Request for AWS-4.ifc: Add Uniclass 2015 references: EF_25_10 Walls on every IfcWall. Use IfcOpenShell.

First a look at what the model holds.

```python
import ifcopenshell

model = ifcopenshell.open("AWS-4.ifc")
print(model.schema)
print("classifications:", [c.Name for c in model.by_type("IfcClassification")])
for ifc_class in ("IfcDoor", "IfcRoof", "IfcStair", "IfcWall", "IfcWindow"):
    print(ifc_class, len(model.by_type(ifc_class)))
```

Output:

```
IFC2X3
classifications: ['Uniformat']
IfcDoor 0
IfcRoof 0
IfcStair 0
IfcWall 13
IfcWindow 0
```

```python
import ifcopenshell
import ifcopenshell.api.classification

model = ifcopenshell.open("AWS-4.ifc")

# IFC2X3 requires Source and Edition and has no link from the project to the system.
system = model.create_entity("IfcClassification", Source="NBS", Edition="2015", Name="Uniclass 2015")

codes = {
    "IfcWall": ("EF_25_10", "Walls"),
}
for ifc_class, (code, name) in codes.items():
    products = model.by_type(ifc_class)
    ifcopenshell.api.classification.add_reference(
        model, products=products, classification=system, identification=code, name=name
    )
    print(code, len(products))

model.write("AWS-4_edited.ifc")
```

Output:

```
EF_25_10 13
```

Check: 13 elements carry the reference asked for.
